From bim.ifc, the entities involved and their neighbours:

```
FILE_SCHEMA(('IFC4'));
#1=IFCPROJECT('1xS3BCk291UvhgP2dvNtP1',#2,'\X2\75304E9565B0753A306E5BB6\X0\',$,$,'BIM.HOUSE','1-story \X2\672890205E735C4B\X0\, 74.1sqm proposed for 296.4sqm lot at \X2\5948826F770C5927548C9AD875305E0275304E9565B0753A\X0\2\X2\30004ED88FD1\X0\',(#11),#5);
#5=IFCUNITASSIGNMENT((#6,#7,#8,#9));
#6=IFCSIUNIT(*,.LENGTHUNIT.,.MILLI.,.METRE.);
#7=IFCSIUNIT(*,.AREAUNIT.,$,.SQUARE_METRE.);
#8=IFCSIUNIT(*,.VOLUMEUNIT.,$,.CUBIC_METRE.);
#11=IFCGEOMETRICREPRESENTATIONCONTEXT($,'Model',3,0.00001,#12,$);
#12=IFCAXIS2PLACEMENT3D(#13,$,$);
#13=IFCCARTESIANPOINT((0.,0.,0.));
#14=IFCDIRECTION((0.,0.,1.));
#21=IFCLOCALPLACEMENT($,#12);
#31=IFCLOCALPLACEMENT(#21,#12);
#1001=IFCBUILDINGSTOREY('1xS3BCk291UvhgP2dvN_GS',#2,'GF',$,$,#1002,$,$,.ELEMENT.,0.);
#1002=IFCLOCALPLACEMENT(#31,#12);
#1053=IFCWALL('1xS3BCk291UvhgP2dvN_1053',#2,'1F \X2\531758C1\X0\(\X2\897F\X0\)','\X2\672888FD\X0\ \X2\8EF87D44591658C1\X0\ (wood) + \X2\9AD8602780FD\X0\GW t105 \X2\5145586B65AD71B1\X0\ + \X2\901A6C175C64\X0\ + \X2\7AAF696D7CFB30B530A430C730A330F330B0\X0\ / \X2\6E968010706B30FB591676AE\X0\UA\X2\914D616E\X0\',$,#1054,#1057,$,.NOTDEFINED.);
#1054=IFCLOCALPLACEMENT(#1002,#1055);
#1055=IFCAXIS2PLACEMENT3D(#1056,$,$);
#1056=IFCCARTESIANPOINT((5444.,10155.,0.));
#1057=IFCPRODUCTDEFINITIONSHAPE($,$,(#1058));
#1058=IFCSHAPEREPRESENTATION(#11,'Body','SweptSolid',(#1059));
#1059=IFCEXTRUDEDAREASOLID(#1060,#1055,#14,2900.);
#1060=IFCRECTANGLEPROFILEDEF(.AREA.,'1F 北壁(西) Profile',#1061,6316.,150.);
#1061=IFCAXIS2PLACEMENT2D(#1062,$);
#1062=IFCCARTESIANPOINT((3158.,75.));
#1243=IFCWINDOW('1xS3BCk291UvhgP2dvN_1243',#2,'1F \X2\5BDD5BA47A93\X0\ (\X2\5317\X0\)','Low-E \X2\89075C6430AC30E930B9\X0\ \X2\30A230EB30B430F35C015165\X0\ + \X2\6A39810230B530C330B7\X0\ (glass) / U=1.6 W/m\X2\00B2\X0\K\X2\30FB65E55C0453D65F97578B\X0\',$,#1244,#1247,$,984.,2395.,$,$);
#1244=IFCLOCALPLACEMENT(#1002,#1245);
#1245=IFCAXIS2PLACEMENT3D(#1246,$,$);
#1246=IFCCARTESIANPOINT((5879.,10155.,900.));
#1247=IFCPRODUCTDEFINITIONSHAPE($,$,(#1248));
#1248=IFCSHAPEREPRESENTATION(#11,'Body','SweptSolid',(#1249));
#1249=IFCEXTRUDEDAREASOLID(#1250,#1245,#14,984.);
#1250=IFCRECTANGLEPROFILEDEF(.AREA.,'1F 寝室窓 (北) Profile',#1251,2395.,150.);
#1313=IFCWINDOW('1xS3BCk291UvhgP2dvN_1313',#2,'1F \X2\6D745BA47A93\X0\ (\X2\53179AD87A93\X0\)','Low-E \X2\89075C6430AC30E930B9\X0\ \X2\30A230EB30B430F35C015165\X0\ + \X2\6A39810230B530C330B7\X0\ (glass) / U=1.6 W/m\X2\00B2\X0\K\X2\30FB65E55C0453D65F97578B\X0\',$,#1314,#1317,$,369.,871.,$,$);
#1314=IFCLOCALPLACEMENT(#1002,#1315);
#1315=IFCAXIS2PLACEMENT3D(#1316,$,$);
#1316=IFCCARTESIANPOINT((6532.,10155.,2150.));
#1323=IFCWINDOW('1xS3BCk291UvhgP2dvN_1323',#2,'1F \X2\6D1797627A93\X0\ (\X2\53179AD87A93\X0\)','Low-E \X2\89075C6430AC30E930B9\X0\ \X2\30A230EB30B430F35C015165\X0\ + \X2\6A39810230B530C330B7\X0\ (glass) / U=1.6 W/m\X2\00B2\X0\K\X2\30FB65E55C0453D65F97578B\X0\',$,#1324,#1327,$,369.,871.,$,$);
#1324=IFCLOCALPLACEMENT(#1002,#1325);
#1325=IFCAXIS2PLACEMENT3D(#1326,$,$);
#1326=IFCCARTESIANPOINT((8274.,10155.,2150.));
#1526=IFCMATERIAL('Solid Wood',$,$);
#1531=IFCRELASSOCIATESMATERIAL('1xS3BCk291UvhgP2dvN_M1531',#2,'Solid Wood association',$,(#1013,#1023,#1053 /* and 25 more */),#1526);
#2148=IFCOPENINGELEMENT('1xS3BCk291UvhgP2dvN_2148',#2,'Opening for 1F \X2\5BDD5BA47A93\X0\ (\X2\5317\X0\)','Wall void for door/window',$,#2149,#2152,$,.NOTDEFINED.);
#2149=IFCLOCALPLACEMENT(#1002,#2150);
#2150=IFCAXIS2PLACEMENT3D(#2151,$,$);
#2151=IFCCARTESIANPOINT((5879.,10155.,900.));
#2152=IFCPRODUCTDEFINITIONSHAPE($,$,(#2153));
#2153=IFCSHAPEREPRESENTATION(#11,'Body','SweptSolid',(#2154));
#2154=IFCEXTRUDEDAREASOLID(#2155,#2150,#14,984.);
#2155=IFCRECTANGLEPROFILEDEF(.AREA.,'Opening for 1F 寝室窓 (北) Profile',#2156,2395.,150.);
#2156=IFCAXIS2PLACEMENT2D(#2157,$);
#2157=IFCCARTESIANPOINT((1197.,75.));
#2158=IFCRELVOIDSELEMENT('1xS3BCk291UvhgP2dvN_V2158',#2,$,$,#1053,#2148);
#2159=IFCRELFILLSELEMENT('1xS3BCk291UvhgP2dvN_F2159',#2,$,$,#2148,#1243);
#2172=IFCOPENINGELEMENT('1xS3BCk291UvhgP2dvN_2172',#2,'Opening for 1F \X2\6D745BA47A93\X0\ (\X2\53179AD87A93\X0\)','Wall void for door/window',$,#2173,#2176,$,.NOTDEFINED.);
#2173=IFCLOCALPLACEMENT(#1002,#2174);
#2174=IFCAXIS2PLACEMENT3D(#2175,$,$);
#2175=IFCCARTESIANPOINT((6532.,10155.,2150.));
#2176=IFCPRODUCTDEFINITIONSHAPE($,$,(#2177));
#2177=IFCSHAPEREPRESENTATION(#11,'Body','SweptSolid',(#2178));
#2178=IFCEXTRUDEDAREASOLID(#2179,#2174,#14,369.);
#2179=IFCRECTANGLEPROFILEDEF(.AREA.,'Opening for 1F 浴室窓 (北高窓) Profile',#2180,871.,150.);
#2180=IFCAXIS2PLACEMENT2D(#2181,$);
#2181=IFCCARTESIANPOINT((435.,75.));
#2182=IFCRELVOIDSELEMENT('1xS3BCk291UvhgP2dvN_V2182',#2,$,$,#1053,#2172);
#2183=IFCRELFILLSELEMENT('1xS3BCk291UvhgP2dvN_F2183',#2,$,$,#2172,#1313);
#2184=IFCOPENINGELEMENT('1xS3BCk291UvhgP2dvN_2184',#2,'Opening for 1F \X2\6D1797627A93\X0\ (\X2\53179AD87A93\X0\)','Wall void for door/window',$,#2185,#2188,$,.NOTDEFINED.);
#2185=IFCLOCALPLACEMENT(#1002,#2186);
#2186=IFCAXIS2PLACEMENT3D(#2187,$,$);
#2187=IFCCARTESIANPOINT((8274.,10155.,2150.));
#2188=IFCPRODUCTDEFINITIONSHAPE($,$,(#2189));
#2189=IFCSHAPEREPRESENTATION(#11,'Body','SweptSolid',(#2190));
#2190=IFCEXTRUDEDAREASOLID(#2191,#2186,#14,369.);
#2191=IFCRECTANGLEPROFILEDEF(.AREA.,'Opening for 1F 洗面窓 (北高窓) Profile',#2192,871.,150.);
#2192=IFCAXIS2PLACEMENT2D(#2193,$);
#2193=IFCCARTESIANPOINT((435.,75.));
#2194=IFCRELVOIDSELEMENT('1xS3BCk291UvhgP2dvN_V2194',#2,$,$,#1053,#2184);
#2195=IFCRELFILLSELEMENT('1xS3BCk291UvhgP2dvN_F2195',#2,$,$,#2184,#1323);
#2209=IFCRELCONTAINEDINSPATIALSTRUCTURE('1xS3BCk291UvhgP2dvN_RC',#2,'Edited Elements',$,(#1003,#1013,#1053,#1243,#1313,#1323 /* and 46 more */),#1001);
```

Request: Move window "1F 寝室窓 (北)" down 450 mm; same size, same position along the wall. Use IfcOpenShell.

```python
import numpy as np
import ifcopenshell
import ifcopenshell.api.geometry
import ifcopenshell.util.placement
import ifcopenshell.util.unit

model = ifcopenshell.open("bim.ifc")
unit_scale = ifcopenshell.util.unit.calculate_unit_scale(model)

window = model.by_guid("1xS3BCk291UvhgP2dvN_1243")
opening = window.FillsVoids[0].RelatingOpeningElement
dz = -0.45 / unit_scale

shift = np.array([0.0, 0.0, dz])
# The window is not placed relative to its opening, so move both.
for product in (opening, window):
    matrix = ifcopenshell.util.placement.get_local_placement(product.ObjectPlacement)
    matrix[:3, 3] += shift
    ifcopenshell.api.geometry.edit_object_placement(model, product=product, matrix=matrix, is_si=False)

print(f"moved by {dz * unit_scale:+.3f} m")

model.write("bim_v2.ifc")
```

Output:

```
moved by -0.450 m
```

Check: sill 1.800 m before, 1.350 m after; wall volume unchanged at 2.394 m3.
